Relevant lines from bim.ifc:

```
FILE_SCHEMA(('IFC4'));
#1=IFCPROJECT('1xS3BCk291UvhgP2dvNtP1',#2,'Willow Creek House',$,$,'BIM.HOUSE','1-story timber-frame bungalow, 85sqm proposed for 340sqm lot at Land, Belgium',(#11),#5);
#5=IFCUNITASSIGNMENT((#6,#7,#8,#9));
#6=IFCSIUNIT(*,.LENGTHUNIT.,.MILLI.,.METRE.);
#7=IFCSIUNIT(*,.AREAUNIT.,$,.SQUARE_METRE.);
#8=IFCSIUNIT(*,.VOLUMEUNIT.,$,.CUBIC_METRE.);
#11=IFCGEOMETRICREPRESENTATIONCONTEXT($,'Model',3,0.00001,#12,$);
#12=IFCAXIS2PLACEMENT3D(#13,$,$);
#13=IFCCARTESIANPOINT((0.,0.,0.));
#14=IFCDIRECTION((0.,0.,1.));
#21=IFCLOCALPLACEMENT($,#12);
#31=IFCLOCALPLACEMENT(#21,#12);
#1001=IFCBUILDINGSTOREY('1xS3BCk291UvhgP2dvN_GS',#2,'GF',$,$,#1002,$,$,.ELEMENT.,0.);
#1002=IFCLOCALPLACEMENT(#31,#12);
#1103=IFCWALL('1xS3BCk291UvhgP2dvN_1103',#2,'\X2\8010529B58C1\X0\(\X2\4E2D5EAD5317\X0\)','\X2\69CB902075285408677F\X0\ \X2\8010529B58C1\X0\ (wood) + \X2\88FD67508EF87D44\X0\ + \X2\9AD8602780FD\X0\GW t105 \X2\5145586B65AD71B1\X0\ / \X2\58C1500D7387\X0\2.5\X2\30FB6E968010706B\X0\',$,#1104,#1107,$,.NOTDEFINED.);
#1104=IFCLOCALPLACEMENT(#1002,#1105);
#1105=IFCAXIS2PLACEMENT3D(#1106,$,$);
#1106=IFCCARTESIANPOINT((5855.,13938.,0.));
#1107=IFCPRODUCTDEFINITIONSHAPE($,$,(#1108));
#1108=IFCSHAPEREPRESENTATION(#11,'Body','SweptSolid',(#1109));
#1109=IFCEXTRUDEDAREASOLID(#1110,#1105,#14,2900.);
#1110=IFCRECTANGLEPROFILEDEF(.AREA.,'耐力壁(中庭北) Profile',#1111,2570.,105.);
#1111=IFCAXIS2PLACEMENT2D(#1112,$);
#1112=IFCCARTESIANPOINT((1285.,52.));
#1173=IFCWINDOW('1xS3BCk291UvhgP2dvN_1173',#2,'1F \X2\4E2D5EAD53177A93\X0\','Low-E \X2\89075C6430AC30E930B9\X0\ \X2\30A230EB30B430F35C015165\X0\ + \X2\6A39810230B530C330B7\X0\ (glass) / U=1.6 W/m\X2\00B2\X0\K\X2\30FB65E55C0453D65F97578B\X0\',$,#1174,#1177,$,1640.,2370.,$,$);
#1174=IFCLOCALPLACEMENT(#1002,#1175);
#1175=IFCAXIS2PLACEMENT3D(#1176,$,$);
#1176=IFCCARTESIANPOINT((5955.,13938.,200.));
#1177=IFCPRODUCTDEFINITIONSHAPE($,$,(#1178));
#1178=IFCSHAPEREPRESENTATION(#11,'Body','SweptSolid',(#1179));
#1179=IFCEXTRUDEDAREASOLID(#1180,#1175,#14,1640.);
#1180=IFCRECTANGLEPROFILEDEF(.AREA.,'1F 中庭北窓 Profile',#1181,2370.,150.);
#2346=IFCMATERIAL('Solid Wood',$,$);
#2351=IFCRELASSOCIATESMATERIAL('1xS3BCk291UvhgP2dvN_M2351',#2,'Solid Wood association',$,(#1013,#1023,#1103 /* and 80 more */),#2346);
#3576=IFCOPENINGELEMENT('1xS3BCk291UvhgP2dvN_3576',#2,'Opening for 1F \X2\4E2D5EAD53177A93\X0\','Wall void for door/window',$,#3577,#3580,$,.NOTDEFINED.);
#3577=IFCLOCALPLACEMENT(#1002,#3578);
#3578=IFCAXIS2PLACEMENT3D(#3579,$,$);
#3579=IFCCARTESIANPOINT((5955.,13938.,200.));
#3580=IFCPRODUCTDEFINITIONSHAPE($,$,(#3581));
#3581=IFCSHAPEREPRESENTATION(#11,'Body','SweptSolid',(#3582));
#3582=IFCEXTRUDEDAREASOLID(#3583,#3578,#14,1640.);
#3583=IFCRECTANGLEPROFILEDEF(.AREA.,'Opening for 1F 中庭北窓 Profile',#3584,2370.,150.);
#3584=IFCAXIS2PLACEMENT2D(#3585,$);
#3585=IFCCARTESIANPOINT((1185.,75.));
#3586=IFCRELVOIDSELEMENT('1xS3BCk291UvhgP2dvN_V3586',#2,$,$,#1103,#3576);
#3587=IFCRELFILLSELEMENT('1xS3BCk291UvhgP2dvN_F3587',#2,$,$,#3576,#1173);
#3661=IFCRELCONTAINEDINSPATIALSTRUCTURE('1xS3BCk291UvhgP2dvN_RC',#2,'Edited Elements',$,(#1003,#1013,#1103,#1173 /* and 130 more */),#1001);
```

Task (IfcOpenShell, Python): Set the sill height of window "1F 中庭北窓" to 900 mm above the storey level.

```python
import numpy as np
import ifcopenshell
import ifcopenshell.api.geometry
import ifcopenshell.geom
import ifcopenshell.util.element
import ifcopenshell.util.placement
import ifcopenshell.util.shape
import ifcopenshell.util.unit

model = ifcopenshell.open("bim.ifc")
unit_scale = ifcopenshell.util.unit.calculate_unit_scale(model)

window = model.by_guid("1xS3BCk291UvhgP2dvN_1173")
opening = window.FillsVoids[0].RelatingOpeningElement
storey = ifcopenshell.util.element.get_container(window, ifc_class="IfcBuildingStorey")
level = ifcopenshell.util.placement.get_local_placement(storey.ObjectPlacement)[2, 3]

# The opening's origin need not be at the sill, so measure its lowest point.
shape = ifcopenshell.geom.create_shape(ifcopenshell.geom.settings(), opening)
bottom = ifcopenshell.util.shape.get_shape_bottom_elevation(shape, shape.geometry) / unit_scale
dz = level + 900.0 - bottom

shift = np.array([0.0, 0.0, dz])
# The window is not placed relative to its opening, so move both.
for product in (opening, window):
    matrix = ifcopenshell.util.placement.get_local_placement(product.ObjectPlacement)
    matrix[:3, 3] += shift
    ifcopenshell.api.geometry.edit_object_placement(model, product=product, matrix=matrix, is_si=False)

print(f"moved by {dz * unit_scale:+.3f} m")

model.write("bim-out.ifc")
```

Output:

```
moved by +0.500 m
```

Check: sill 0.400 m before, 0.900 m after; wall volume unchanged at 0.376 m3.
